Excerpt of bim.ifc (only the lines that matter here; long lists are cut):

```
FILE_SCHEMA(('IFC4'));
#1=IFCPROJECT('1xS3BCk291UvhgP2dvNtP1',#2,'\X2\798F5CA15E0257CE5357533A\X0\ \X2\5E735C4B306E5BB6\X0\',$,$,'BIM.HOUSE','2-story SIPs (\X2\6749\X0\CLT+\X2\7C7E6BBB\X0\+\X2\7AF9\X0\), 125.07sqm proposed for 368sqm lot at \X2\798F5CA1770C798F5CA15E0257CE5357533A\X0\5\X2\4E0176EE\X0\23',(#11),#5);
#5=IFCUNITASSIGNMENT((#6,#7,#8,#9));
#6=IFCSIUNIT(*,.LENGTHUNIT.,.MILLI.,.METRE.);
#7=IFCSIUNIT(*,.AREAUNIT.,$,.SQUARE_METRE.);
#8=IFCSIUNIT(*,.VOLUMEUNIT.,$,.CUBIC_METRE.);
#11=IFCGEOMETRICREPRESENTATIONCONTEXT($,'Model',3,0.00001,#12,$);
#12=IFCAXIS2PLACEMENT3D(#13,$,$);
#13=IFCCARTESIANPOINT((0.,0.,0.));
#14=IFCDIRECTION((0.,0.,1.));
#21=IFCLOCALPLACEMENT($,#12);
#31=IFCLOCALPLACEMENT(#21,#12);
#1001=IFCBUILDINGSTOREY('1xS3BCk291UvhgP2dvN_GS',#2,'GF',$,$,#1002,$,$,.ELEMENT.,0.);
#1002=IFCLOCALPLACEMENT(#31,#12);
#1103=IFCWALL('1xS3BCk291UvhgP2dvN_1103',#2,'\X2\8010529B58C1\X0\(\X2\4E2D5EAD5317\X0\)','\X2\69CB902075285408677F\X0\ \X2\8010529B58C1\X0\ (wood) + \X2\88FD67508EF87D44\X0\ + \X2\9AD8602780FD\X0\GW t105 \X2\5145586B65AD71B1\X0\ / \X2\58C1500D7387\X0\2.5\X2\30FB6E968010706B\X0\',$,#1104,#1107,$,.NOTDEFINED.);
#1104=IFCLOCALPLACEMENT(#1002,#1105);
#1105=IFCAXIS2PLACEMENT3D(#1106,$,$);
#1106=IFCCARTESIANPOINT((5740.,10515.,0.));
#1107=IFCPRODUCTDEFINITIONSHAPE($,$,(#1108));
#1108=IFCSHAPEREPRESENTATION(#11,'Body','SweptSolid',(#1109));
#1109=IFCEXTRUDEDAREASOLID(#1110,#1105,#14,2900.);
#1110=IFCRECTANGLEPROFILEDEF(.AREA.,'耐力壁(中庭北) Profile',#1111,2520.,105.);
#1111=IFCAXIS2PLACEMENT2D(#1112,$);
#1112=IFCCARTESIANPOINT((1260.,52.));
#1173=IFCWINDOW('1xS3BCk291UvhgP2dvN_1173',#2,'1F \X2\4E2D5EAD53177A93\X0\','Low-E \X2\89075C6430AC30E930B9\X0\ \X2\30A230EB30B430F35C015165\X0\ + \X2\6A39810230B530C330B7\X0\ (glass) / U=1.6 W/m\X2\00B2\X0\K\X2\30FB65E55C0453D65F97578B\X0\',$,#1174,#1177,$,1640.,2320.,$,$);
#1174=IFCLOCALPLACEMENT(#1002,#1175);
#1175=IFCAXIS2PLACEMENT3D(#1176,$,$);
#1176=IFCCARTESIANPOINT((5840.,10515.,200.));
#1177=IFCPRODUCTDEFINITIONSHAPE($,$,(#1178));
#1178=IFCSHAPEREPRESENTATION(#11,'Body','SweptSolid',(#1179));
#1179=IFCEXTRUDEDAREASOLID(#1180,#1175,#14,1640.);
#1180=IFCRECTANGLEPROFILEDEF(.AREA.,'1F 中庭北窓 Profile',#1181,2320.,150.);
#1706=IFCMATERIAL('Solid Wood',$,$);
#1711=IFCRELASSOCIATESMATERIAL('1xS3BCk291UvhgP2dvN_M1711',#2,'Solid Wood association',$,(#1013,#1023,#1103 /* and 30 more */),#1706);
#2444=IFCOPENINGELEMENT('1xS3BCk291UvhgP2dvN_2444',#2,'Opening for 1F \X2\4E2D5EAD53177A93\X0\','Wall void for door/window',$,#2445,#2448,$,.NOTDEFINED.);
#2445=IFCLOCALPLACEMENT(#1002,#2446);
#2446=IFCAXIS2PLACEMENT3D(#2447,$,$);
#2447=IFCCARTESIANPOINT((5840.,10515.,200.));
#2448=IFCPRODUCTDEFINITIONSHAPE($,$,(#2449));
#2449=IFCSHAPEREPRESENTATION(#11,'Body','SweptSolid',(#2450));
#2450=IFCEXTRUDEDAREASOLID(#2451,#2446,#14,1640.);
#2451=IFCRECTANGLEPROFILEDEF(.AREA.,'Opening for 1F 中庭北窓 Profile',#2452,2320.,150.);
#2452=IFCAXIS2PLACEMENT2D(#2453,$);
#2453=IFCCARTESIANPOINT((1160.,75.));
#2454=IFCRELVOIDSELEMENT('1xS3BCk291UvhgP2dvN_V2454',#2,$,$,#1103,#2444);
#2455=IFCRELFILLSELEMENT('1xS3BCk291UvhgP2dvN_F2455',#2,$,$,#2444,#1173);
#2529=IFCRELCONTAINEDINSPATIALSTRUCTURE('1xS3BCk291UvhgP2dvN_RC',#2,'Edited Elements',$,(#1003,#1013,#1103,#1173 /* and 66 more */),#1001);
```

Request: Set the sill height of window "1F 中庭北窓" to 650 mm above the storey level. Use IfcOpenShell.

```python
import numpy as np
import ifcopenshell
import ifcopenshell.api.geometry
import ifcopenshell.geom
import ifcopenshell.util.element
import ifcopenshell.util.placement
import ifcopenshell.util.shape
import ifcopenshell.util.unit

model = ifcopenshell.open("bim.ifc")
unit_scale = ifcopenshell.util.unit.calculate_unit_scale(model)

window = model.by_id(1173)
opening = window.FillsVoids[0].RelatingOpeningElement
storey = ifcopenshell.util.element.get_container(window, ifc_class="IfcBuildingStorey")
level = ifcopenshell.util.placement.get_local_placement(storey.ObjectPlacement)[2, 3]

# The opening's origin need not be at the sill, so measure its lowest point.
shape = ifcopenshell.geom.create_shape(ifcopenshell.geom.settings(), opening)
bottom = ifcopenshell.util.shape.get_shape_bottom_elevation(shape, shape.geometry) / unit_scale
dz = level + 0.65 / unit_scale - bottom

shift = np.array([0.0, 0.0, dz])
# The window is not placed relative to its opening, so move both.
for product in (opening, window):
    matrix = ifcopenshell.util.placement.get_local_placement(product.ObjectPlacement)
    matrix[:3, 3] += shift
    ifcopenshell.api.geometry.edit_object_placement(model, product=product, matrix=matrix, is_si=False)

print(f"moved by {dz * unit_scale:+.3f} m")

model.write("bim_updated.ifc")
```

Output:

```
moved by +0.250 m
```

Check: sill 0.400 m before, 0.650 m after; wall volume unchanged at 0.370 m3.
